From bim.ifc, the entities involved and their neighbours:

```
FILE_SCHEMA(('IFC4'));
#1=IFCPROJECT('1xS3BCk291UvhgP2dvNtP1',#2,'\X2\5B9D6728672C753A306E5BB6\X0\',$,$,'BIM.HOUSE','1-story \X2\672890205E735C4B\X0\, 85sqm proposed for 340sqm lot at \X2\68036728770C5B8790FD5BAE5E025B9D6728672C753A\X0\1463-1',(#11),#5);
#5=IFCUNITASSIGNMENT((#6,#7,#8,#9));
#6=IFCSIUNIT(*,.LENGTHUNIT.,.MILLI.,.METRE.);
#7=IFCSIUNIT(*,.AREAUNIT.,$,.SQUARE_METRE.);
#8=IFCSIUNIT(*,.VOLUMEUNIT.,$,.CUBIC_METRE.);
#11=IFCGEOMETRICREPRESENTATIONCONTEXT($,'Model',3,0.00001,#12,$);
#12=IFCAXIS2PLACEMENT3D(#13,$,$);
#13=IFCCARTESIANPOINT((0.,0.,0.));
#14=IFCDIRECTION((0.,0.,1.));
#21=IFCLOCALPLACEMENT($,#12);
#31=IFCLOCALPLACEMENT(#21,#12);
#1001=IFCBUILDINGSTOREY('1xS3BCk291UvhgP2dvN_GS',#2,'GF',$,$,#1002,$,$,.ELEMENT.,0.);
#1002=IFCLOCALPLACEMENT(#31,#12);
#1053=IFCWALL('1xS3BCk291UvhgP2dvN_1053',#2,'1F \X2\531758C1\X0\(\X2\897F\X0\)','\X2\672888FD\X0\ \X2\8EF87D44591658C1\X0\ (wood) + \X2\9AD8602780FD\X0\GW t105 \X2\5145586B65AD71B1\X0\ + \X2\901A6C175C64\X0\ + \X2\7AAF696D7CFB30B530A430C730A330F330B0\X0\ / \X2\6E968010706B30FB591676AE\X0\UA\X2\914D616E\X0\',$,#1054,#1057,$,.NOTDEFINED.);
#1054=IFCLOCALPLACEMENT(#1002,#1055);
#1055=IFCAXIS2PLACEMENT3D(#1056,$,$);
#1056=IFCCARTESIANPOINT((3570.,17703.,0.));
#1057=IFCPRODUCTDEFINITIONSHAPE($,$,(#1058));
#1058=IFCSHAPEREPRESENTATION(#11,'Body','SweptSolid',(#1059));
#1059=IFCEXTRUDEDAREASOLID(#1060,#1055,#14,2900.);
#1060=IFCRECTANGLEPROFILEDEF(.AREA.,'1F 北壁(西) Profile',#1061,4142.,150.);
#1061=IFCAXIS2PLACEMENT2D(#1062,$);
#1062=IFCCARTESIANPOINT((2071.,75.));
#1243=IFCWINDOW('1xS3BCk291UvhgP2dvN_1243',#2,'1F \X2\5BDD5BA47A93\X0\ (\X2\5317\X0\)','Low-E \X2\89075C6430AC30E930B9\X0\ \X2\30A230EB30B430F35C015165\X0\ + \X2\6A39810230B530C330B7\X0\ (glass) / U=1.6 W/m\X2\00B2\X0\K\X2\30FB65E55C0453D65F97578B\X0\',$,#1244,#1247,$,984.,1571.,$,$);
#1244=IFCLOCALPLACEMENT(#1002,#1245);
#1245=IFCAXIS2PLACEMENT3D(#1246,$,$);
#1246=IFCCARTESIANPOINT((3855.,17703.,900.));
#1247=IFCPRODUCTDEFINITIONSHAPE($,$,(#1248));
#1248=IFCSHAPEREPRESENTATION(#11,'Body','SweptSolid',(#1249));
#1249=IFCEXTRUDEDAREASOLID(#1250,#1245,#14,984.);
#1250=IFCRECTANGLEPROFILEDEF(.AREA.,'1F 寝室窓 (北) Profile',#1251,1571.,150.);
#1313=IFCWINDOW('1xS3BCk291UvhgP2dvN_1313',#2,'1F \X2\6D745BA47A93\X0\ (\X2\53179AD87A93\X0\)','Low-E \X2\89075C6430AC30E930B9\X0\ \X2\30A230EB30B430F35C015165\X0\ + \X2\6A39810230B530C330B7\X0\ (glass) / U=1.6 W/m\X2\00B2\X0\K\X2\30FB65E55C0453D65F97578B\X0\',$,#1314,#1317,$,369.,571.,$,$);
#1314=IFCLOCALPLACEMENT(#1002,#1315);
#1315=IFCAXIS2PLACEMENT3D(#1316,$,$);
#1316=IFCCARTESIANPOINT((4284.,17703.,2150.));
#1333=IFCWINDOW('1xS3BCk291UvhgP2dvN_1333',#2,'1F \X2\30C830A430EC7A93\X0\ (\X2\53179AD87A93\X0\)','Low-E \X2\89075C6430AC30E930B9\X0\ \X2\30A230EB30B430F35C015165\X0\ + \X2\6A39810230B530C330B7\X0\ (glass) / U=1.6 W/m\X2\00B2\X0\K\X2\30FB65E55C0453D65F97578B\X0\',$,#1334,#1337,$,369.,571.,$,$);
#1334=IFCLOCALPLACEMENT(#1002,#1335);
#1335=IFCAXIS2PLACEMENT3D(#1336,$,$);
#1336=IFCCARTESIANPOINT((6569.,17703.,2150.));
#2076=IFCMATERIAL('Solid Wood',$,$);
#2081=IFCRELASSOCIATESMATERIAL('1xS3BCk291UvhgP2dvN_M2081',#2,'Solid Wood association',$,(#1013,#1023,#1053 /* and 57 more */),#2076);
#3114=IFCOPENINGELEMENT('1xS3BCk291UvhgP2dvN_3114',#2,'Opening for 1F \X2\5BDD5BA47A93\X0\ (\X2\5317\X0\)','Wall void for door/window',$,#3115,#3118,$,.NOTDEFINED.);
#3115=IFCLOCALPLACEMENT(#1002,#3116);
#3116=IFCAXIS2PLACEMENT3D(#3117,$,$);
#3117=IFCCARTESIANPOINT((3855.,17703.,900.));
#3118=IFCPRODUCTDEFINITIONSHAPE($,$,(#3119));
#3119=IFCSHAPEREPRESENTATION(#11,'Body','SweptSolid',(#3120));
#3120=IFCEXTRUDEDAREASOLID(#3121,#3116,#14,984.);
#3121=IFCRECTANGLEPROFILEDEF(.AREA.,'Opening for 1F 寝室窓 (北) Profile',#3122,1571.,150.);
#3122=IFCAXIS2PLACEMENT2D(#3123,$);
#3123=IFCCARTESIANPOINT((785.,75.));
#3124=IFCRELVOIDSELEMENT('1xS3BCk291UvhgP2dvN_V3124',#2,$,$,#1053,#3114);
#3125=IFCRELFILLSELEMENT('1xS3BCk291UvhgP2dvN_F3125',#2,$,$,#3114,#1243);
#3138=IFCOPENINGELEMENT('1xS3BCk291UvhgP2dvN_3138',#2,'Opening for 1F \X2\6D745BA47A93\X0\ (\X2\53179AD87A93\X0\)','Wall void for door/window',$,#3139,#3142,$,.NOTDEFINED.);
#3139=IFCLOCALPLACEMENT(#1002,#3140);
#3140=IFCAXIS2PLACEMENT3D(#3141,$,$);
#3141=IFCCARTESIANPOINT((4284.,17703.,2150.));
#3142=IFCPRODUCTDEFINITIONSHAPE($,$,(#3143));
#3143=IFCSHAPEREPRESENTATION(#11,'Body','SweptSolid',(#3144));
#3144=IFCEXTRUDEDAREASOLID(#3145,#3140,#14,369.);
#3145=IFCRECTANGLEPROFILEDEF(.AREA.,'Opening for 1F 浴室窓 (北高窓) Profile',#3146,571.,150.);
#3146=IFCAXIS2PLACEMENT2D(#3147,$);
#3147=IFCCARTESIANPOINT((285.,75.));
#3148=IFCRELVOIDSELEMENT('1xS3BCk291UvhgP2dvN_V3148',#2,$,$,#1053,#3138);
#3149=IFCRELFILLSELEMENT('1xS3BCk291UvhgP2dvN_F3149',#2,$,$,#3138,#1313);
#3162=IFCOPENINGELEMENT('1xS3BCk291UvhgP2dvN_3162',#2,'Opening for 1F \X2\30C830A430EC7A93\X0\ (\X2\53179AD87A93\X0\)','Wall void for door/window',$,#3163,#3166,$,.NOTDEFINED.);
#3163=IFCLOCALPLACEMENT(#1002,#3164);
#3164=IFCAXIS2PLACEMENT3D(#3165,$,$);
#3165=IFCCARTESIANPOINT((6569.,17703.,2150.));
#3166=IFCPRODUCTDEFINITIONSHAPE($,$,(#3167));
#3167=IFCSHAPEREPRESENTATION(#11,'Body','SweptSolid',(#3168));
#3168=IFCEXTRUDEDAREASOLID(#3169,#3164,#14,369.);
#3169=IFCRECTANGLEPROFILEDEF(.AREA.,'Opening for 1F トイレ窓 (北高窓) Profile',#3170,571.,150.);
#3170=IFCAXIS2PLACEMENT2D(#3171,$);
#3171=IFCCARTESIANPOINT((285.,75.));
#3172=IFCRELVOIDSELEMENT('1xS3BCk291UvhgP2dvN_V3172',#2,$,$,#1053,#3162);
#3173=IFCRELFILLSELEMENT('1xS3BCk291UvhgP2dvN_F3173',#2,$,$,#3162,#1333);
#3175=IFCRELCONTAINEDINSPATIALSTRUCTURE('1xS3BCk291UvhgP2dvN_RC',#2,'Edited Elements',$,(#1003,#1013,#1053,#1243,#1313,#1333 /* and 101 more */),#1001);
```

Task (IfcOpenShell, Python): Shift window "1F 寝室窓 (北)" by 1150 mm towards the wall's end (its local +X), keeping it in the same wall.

```python
import ifcopenshell
import ifcopenshell.api.geometry
import ifcopenshell.util.placement
import ifcopenshell.util.unit

model = ifcopenshell.open("bim.ifc")
unit_scale = ifcopenshell.util.unit.calculate_unit_scale(model)

window = model.by_guid("1xS3BCk291UvhgP2dvN_1243")
opening = window.FillsVoids[0].RelatingOpeningElement
wall = opening.VoidsElements[0].RelatingBuildingElement

wall_matrix = ifcopenshell.util.placement.get_local_placement(wall.ObjectPlacement)
shift = wall_matrix[:3, 0] * 1.15 / unit_scale
before = ifcopenshell.util.placement.get_local_placement(window.ObjectPlacement)[:3, 3].copy()

# The window is not placed relative to its opening, so move both.
for product in (opening, window):
    matrix = ifcopenshell.util.placement.get_local_placement(product.ObjectPlacement)
    matrix[:3, 3] += shift
    ifcopenshell.api.geometry.edit_object_placement(model, product=product, matrix=matrix, is_si=False)

after = ifcopenshell.util.placement.get_local_placement(window.ObjectPlacement)[:3, 3]
print("window moved by", (after - before).round(3) + 0.0)

model.write("bim_updated.ifc")
```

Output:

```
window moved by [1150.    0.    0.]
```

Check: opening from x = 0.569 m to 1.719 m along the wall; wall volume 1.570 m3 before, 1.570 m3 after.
